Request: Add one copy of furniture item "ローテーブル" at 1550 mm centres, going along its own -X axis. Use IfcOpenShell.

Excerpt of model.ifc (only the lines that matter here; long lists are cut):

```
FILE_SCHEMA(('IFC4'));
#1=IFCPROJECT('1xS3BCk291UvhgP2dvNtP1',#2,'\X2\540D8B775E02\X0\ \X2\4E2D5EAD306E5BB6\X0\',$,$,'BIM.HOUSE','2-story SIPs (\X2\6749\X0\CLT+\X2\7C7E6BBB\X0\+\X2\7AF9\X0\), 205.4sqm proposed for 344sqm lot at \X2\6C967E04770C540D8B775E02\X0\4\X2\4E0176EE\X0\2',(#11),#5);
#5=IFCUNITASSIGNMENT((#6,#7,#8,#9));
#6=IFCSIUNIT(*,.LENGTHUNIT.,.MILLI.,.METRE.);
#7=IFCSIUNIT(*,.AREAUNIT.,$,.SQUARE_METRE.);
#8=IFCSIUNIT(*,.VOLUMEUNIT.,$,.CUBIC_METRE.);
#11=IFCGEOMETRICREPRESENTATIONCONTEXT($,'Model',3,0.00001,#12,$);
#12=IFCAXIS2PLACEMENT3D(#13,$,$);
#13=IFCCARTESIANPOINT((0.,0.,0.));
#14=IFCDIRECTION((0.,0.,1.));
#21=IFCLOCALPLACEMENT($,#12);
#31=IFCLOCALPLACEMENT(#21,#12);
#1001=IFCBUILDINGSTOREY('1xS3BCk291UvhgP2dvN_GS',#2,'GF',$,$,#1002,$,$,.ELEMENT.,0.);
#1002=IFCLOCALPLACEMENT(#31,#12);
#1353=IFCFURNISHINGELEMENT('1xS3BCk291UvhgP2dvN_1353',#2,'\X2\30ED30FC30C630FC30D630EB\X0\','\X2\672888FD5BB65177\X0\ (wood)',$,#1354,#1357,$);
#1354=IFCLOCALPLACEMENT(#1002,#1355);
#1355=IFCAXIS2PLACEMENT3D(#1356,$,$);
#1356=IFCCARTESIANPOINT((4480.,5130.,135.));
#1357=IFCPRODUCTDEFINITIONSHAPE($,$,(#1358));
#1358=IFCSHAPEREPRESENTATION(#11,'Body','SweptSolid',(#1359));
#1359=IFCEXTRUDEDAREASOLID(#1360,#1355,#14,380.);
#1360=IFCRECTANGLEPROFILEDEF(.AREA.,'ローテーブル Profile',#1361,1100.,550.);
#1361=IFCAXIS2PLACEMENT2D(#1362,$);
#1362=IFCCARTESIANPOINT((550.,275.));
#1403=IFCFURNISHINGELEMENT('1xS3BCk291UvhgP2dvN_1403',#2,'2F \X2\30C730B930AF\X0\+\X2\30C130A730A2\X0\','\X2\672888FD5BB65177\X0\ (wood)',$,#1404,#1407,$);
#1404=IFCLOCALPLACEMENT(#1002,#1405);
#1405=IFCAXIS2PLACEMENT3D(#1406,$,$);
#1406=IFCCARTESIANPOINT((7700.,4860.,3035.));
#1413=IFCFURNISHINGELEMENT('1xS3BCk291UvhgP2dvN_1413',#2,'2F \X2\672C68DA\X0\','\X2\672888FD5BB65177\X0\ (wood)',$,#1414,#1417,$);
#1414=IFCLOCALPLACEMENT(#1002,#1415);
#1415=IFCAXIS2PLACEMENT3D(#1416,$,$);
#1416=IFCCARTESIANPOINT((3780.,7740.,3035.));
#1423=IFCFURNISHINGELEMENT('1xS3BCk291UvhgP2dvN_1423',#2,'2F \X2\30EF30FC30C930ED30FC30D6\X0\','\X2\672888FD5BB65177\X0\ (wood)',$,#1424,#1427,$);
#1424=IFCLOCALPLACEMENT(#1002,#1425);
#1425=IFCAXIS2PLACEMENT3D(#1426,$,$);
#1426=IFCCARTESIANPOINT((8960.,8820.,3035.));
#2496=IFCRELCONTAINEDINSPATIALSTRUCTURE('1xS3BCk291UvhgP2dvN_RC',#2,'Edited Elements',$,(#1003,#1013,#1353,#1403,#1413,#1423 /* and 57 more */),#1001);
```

```python
import ifcopenshell
import ifcopenshell.api.geometry
import ifcopenshell.api.root
import ifcopenshell.util.element
import ifcopenshell.util.placement
import ifcopenshell.util.unit

model = ifcopenshell.open("model.ifc")
unit_scale = ifcopenshell.util.unit.calculate_unit_scale(model)


def reuse_history(source, copy):
    """copy_class also copies each property set's owner history, people and application; keep the originals."""
    for rel in copy.IsDefinedBy:
        if rel.is_a("IfcRelDefinesByProperties") and (history := rel.RelatingPropertyDefinition.OwnerHistory):
            rel.RelatingPropertyDefinition.OwnerHistory = source.OwnerHistory
            ifcopenshell.util.element.remove_deep2(model, history)


source = model.by_guid("1xS3BCk291UvhgP2dvN_1353")
base = ifcopenshell.util.placement.get_local_placement(source.ObjectPlacement)
step = -base[:3, 0] * 1.55 / unit_scale

for i in range(1, 2):
    copy = ifcopenshell.api.root.copy_class(model, product=source)
    copy.Representation = ifcopenshell.util.element.copy_deep(
        model, source.Representation, exclude=["IfcGeometricRepresentationContext", "IfcRepresentationMap"]
    )
    reuse_history(source, copy)
    matrix = base.copy()
    matrix[:3, 3] += i * step
    print("added at", matrix[:3, 3].round(3) + 0.0)
    ifcopenshell.api.geometry.edit_object_placement(model, product=copy, matrix=matrix, is_si=False)

model.write("model_updated.ifc")
```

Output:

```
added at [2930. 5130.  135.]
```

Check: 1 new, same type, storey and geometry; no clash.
